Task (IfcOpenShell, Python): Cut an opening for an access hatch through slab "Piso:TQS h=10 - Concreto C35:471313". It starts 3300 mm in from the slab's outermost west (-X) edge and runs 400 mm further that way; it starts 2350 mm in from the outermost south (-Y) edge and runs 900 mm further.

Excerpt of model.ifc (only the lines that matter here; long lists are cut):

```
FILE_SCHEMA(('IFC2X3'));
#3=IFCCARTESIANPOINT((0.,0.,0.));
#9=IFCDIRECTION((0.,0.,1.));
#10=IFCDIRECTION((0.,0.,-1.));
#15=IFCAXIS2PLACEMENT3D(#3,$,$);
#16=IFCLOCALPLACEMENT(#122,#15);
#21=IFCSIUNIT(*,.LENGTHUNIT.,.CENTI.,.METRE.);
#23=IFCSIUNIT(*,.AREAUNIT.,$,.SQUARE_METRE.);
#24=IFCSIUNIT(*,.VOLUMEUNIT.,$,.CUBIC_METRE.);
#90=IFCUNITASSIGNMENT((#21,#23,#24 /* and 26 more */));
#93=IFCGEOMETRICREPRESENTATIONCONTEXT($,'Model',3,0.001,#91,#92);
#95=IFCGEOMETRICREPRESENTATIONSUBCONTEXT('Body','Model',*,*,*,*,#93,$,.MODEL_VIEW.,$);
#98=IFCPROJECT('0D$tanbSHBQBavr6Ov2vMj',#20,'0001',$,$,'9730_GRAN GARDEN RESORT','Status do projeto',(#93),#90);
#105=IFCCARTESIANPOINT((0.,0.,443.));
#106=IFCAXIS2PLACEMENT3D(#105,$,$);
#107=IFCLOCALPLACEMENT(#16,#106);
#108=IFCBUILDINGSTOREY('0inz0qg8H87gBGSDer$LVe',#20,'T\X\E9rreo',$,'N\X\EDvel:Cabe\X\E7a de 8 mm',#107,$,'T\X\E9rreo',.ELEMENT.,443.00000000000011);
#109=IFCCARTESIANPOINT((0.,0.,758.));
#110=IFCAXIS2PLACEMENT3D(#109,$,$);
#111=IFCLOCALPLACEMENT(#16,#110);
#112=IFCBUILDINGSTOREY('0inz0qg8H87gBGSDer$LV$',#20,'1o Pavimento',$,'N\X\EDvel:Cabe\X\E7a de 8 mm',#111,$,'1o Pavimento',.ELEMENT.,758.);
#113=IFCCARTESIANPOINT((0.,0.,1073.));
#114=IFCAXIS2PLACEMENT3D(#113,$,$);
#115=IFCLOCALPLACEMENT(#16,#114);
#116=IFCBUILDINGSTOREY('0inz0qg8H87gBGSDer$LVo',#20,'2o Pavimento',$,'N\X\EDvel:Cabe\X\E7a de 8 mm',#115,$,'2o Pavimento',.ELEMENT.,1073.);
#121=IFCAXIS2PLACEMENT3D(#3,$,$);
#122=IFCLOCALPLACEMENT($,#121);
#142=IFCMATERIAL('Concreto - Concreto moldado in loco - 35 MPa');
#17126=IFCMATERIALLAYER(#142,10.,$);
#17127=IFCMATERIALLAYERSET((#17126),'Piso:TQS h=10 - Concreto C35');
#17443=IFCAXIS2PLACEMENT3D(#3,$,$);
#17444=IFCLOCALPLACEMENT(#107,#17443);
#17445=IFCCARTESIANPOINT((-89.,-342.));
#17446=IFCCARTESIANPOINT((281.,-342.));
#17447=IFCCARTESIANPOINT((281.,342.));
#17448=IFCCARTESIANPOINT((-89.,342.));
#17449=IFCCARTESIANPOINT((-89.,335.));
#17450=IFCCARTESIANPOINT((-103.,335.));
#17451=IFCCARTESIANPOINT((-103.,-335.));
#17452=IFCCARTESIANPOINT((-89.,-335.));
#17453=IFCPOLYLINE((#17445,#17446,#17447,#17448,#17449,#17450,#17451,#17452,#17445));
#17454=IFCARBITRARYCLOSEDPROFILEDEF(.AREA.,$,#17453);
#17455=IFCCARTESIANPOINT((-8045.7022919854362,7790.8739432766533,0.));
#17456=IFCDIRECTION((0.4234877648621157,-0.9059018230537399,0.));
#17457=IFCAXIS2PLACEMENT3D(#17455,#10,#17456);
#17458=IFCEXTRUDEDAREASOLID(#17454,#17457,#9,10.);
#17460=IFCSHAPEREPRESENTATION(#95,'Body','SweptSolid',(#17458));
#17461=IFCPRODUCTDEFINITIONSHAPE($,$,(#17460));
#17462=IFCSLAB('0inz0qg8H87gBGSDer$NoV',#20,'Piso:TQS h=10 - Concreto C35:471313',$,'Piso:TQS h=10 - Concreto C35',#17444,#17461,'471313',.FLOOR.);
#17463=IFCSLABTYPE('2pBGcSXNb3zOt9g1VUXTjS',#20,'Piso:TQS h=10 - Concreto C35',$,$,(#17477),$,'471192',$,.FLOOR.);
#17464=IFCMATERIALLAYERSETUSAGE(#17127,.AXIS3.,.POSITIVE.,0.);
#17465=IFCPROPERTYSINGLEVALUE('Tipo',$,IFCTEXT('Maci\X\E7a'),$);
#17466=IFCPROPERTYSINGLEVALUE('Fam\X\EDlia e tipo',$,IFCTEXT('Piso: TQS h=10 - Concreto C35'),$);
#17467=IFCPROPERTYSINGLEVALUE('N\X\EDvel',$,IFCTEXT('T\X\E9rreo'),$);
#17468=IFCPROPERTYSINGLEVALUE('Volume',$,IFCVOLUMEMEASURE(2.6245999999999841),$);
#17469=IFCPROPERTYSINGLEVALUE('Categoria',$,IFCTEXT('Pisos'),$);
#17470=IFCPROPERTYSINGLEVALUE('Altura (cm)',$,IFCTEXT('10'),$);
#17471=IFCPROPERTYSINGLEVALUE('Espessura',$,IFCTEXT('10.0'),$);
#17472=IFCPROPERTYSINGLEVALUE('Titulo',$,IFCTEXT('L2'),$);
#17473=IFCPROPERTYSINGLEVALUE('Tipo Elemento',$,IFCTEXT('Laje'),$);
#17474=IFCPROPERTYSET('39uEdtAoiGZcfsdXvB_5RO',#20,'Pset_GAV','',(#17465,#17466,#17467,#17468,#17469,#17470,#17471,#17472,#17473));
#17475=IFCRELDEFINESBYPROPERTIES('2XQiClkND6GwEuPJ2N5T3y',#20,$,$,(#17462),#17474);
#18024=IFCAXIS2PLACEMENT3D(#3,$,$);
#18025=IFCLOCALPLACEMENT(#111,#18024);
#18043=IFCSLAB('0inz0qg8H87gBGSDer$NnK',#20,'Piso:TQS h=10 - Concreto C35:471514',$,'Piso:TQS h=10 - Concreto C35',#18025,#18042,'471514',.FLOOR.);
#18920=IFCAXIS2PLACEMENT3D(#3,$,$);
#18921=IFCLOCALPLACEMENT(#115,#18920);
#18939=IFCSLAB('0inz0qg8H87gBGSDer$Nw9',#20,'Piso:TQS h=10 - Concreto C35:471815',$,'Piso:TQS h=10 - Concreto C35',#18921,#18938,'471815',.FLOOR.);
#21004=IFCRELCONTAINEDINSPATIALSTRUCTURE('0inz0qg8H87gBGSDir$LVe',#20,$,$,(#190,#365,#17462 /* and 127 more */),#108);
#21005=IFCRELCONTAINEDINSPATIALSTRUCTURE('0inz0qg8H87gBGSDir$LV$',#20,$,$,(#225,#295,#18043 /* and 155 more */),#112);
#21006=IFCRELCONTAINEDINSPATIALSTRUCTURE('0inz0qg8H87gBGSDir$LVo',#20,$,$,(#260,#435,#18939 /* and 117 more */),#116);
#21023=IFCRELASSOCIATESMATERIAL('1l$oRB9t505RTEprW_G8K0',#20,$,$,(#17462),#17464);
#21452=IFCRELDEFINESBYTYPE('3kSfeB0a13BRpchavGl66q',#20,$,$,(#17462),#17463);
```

```python
import numpy as np
import ifcopenshell
import ifcopenshell.api.feature
import ifcopenshell.api.geometry
import ifcopenshell.api.pset
import ifcopenshell.api.root
import ifcopenshell.geom
import ifcopenshell.util.element
import ifcopenshell.util.placement
import ifcopenshell.util.representation
import ifcopenshell.util.shape
import ifcopenshell.util.unit

model = ifcopenshell.open("model.ifc")
unit_scale = ifcopenshell.util.unit.calculate_unit_scale(model)
volume_scale = ifcopenshell.util.unit.calculate_unit_scale(model, "VOLUMEUNIT")
settings = ifcopenshell.geom.settings()


def volume(element):
    """Net volume in cubic metres, openings subtracted."""
    shape = ifcopenshell.geom.create_shape(settings, element)
    return ifcopenshell.util.shape.get_volume(shape.geometry)


slab = model.by_guid("0inz0qg8H87gBGSDer$NoV")
before = volume(slab)

# Extent in the slab's own axes, in metres. The edges named are its -X and -Y sides.
slab_shape = ifcopenshell.geom.create_shape(settings, slab)
vertices = ifcopenshell.util.shape.get_vertices(slab_shape.geometry)
x_min, y_min, bottom = vertices.min(axis=0)
top = vertices[:, 2].max()

opening = ifcopenshell.api.root.create_entity(model, ifc_class="IfcOpeningElement", name="Access hatch opening")
context = ifcopenshell.util.representation.get_context(model, "Model", "Body", "MODEL_VIEW")
width, depth = 0.4, 0.9
outline = [(0.0, 0.0), (width, 0.0), (width, depth), (0.0, depth), (0.0, 0.0)]
# Overshoot both faces by 50 mm so the cut is clean.
shape = ifcopenshell.api.geometry.add_slab_representation(
    model, context=context, depth=top - bottom + 0.1, polyline=outline
)
ifcopenshell.api.geometry.assign_representation(model, product=opening, representation=shape)

matrix = ifcopenshell.util.placement.get_local_placement(slab.ObjectPlacement)
matrix[:, 3] = matrix @ np.append(np.array([x_min + 3.3, y_min + 2.35, bottom - 0.05]) / unit_scale, 1.0)
ifcopenshell.api.geometry.edit_object_placement(model, product=opening, matrix=matrix, is_si=False)
ifcopenshell.api.feature.add_feature(model, feature=opening, element=slab)

after = volume(slab)

# Update the slab's stored quantities.
pset = model.by_id(ifcopenshell.util.element.get_pset(slab, "Pset_GAV", should_inherit=False)["id"])
ifcopenshell.api.pset.edit_pset(model, pset=pset, properties={
    "Volume": model.create_entity("IfcVolumeMeasure", after / volume_scale),
})

print(f"slab volume {before:.3f} -> {after:.3f} m3")

model.write("model-out.ifc")
```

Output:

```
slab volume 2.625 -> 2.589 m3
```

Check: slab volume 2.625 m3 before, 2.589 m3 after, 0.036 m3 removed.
